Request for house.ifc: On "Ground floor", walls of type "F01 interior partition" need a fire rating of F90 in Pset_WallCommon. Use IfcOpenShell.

First a look at what the model holds.

```python
import ifcopenshell
import ifcopenshell.util.element

model = ifcopenshell.open("house.ifc")
print(model.schema)
storey = next(s for s in model.by_type("IfcBuildingStorey") if s.Name == "Ground floor")
walls = [e for e in ifcopenshell.util.element.get_decomposition(storey) if e.is_a("IfcWall")]
seen = {}
for e in walls:
    element_type = ifcopenshell.util.element.get_type(e)
    key = (element_type.Name if element_type != e and element_type else None, ifcopenshell.util.element.get_pset(e, "Pset_WallCommon", "FireRating"))
    seen[key] = seen.get(key, 0) + 1
for (name, value), count in sorted(seen.items(), key=str):
    print(count, "x", name, "|", value)
```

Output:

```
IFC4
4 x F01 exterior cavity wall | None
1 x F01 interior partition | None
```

```python
import ifcopenshell
import ifcopenshell.api.pset
import ifcopenshell.util.element

model = ifcopenshell.open("house.ifc")

storey = next(s for s in model.by_type("IfcBuildingStorey") if s.Name == "Ground floor")
walls = [e for e in ifcopenshell.util.element.get_decomposition(storey) if e.is_a("IfcWall")]

count = 0
for e in walls:
    element_type = ifcopenshell.util.element.get_type(e)
    if element_type in (None, e) or element_type.Name != "F01 interior partition":
        continue
    # add_pset returns the element's existing set when there is one.
    pset = ifcopenshell.api.pset.add_pset(model, product=e, name="Pset_WallCommon")
    ifcopenshell.api.pset.edit_pset(model, pset=pset, properties={"FireRating": "F90"})
    count += 1

print(count, "walls updated")

model.write("house_rev.ifc")
```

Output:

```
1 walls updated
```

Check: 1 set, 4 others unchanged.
